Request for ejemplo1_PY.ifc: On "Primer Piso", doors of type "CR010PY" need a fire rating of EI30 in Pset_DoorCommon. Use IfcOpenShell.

First a look at what the model holds.

```python
import ifcopenshell
import ifcopenshell.util.element

model = ifcopenshell.open("ejemplo1_PY.ifc")
print(model.schema)
storey = next(s for s in model.by_type("IfcBuildingStorey") if s.Name == "Primer Piso")
doors = [e for e in ifcopenshell.util.element.get_decomposition(storey) if e.is_a("IfcDoor")]
seen = {}
for e in doors:
    element_type = ifcopenshell.util.element.get_type(e)
    key = (element_type.Name if element_type != e and element_type else None, ifcopenshell.util.element.get_pset(e, "Pset_DoorCommon", "FireRating"))
    seen[key] = seen.get(key, 0) + 1
for (name, value), count in sorted(seen.items(), key=str):
    print(count, "x", name, "|", value)
```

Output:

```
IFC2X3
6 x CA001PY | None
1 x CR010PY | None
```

```python
import ifcopenshell
import ifcopenshell.api.pset
import ifcopenshell.util.element

model = ifcopenshell.open("ejemplo1_PY.ifc")

storey = next(s for s in model.by_type("IfcBuildingStorey") if s.Name == "Primer Piso")
doors = [e for e in ifcopenshell.util.element.get_decomposition(storey) if e.is_a("IfcDoor")]

count = 0
for e in doors:
    element_type = ifcopenshell.util.element.get_type(e)
    if element_type in (None, e) or element_type.Name != "CR010PY":
        continue
    # add_pset returns the element's existing set when there is one.
    pset = ifcopenshell.api.pset.add_pset(model, product=e, name="Pset_DoorCommon")
    ifcopenshell.api.pset.edit_pset(model, pset=pset, properties={"FireRating": "EI30"})
    count += 1

print(count, "doors updated")

model.write("ejemplo1_PY-out.ifc")
```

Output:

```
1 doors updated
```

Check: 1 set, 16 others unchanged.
